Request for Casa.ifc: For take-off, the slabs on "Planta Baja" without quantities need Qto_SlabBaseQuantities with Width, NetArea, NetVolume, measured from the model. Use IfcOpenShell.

First a look at what the model holds.

```python
import ifcopenshell
import ifcopenshell.util.element
import ifcopenshell.util.unit

model = ifcopenshell.open("Casa.ifc")
print(model.schema)
for unit_type in ("LENGTHUNIT", "AREAUNIT", "VOLUMEUNIT"):
    print(unit_type, ifcopenshell.util.unit.calculate_unit_scale(model, unit_type))
storey = next(s for s in model.by_type("IfcBuildingStorey") if s.Name == "Planta Baja")
slabs = [e for e in ifcopenshell.util.element.get_decomposition(storey) if e.is_a("IfcSlab")]
for e in sorted(slabs, key=lambda e: e.id()):
    print(e.id(), e.is_a(), e.Name, list(ifcopenshell.util.element.get_psets(e, qtos_only=True)), sep=" | ")
```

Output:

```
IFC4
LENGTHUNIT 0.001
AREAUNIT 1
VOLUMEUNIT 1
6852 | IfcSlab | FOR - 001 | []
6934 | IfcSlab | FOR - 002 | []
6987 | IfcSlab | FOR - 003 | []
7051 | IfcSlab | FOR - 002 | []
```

```python
import ifcopenshell
import ifcopenshell.api.pset
import ifcopenshell.geom
import ifcopenshell.util.element
import ifcopenshell.util.shape
import ifcopenshell.util.unit

model = ifcopenshell.open("Casa.ifc")
unit_scale = ifcopenshell.util.unit.calculate_unit_scale(model)
area_scale = ifcopenshell.util.unit.calculate_unit_scale(model, "AREAUNIT")
volume_scale = ifcopenshell.util.unit.calculate_unit_scale(model, "VOLUMEUNIT")
settings = ifcopenshell.geom.settings()

storey = next(s for s in model.by_type("IfcBuildingStorey") if s.Name == "Planta Baja")
slabs = [e for e in ifcopenshell.util.element.get_decomposition(storey) if e.is_a("IfcSlab")]

for e in sorted(slabs, key=lambda e: e.id()):
    if ifcopenshell.util.element.get_psets(e, qtos_only=True, should_inherit=False):
        continue
    # Geometry comes back in metres, in the element's own axes.
    shape = ifcopenshell.geom.create_shape(settings, e)
    values = {
        "Width": ifcopenshell.util.shape.get_z(shape.geometry) / unit_scale,
        "NetArea": ifcopenshell.util.shape.get_footprint_area(shape.geometry) / area_scale,
        "NetVolume": ifcopenshell.util.shape.get_volume(shape.geometry) / volume_scale,
    }
    qto = ifcopenshell.api.pset.add_qto(model, product=e, name="Qto_SlabBaseQuantities")
    ifcopenshell.api.pset.edit_qto(model, qto=qto, properties=values)
    print(e.id(), {k: round(v, 3) for k, v in values.items()})

model.write("Casa_rev.ifc")
```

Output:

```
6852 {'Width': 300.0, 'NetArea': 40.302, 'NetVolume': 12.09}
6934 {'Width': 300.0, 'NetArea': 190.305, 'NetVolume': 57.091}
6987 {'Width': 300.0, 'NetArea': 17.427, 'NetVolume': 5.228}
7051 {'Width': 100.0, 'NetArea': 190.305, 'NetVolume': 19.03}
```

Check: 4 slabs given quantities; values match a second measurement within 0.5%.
